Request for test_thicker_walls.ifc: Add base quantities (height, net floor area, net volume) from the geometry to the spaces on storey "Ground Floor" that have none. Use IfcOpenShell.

First a look at what the model holds.

```python
import ifcopenshell
import ifcopenshell.util.element
import ifcopenshell.util.unit

model = ifcopenshell.open("test_thicker_walls.ifc")
print(model.schema)
for unit_type in ("LENGTHUNIT", "AREAUNIT", "VOLUMEUNIT"):
    print(unit_type, ifcopenshell.util.unit.calculate_unit_scale(model, unit_type))
storey = next(s for s in model.by_type("IfcBuildingStorey") if s.Name == "Ground Floor")
spaces = [e for e in ifcopenshell.util.element.get_decomposition(storey) if e.is_a("IfcSpace")]
for e in sorted(spaces, key=lambda e: e.id()):
    print(e.id(), e.is_a(), e.Name, list(ifcopenshell.util.element.get_psets(e, qtos_only=True)), sep=" | ")
```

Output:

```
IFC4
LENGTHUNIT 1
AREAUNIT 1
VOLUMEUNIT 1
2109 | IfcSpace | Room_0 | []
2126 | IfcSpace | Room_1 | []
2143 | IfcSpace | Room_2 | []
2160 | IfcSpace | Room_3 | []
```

```python
import ifcopenshell
import ifcopenshell.api.pset
import ifcopenshell.geom
import ifcopenshell.util.element
import ifcopenshell.util.shape
import ifcopenshell.util.unit

model = ifcopenshell.open("test_thicker_walls.ifc")
unit_scale = ifcopenshell.util.unit.calculate_unit_scale(model)
area_scale = ifcopenshell.util.unit.calculate_unit_scale(model, "AREAUNIT")
volume_scale = ifcopenshell.util.unit.calculate_unit_scale(model, "VOLUMEUNIT")
settings = ifcopenshell.geom.settings()

storey = next(s for s in model.by_type("IfcBuildingStorey") if s.Name == "Ground Floor")
spaces = [e for e in ifcopenshell.util.element.get_decomposition(storey) if e.is_a("IfcSpace")]

for e in sorted(spaces, key=lambda e: e.id()):
    if ifcopenshell.util.element.get_psets(e, qtos_only=True, should_inherit=False):
        continue
    # Geometry comes back in metres, in the element's own axes.
    shape = ifcopenshell.geom.create_shape(settings, e)
    values = {
        "Height": ifcopenshell.util.shape.get_z(shape.geometry) / unit_scale,
        "NetFloorArea": ifcopenshell.util.shape.get_footprint_area(shape.geometry) / area_scale,
        "NetVolume": ifcopenshell.util.shape.get_volume(shape.geometry) / volume_scale,
    }
    qto = ifcopenshell.api.pset.add_qto(model, product=e, name="Qto_SpaceBaseQuantities")
    ifcopenshell.api.pset.edit_qto(model, qto=qto, properties=values)
    print(e.id(), {k: round(v, 3) for k, v in values.items()})

model.write("test_thicker_walls-out.ifc")
```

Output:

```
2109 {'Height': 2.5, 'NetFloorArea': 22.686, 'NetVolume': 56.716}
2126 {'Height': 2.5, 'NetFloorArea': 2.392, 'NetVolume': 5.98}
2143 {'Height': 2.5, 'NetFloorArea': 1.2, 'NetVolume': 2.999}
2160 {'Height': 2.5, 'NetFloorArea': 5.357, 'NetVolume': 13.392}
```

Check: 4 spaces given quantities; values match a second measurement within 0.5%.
